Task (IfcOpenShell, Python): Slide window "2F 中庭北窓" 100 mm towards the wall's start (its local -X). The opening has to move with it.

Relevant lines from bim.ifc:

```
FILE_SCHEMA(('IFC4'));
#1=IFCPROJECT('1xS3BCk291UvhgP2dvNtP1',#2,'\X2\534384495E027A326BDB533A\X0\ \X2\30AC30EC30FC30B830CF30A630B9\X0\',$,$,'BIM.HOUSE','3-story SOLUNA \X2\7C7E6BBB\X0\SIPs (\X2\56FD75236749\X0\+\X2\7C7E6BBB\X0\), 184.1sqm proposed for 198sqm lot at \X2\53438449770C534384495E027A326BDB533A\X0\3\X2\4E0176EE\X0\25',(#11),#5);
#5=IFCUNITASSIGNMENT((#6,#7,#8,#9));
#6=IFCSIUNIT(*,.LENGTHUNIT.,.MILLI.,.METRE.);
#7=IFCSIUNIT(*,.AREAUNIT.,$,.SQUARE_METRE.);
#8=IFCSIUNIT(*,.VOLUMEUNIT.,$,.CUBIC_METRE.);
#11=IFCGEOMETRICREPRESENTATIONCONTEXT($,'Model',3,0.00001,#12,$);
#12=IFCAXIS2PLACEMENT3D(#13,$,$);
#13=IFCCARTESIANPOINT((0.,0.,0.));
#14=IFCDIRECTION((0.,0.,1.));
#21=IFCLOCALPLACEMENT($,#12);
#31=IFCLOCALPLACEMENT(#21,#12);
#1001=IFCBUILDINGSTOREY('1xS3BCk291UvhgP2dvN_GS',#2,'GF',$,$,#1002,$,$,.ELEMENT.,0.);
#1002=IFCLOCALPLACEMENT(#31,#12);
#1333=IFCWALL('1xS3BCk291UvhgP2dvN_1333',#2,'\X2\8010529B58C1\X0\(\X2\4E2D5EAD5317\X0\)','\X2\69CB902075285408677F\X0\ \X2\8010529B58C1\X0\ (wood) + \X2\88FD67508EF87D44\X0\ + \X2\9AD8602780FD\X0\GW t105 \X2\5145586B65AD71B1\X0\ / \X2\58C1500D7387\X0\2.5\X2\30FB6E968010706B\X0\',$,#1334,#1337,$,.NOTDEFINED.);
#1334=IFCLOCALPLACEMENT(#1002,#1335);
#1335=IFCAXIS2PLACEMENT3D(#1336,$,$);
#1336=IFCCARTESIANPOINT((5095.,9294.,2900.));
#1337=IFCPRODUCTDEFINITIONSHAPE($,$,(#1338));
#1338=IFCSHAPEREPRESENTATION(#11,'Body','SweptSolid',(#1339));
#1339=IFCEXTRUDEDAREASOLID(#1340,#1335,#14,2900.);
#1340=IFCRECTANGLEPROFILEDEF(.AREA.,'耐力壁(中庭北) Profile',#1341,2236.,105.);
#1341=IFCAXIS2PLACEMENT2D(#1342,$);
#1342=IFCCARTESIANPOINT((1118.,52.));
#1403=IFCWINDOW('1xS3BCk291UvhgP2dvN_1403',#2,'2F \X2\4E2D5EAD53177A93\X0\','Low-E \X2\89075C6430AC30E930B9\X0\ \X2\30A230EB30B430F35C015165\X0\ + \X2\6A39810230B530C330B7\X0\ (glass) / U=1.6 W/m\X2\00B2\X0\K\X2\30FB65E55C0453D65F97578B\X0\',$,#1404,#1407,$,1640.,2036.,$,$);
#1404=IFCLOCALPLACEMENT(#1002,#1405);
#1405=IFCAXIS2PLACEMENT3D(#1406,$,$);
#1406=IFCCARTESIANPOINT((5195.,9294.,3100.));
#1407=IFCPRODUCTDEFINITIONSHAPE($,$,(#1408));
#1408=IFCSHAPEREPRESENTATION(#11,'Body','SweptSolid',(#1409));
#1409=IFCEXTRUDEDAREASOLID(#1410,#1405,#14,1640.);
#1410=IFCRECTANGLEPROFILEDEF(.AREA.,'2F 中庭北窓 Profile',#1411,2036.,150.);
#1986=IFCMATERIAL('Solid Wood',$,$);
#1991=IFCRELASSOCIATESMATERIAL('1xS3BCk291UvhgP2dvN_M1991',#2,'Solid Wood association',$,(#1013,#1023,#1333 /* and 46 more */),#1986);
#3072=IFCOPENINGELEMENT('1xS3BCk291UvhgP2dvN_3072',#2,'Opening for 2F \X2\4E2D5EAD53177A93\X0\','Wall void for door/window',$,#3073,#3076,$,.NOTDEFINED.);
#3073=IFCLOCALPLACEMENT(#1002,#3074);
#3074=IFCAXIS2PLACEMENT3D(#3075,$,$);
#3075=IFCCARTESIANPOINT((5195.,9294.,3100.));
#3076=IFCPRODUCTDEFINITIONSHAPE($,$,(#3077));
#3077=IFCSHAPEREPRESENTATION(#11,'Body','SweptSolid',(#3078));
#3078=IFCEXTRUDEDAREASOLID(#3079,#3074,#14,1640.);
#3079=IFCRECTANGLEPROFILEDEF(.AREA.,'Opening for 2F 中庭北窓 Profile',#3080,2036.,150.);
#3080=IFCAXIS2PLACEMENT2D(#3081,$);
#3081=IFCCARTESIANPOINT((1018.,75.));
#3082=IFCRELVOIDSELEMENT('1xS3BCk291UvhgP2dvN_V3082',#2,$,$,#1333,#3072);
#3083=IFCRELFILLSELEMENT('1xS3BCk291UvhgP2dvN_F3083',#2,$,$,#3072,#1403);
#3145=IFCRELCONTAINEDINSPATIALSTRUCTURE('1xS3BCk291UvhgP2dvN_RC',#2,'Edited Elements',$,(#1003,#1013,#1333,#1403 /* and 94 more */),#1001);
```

```python
import ifcopenshell
import ifcopenshell.api.geometry
import ifcopenshell.util.placement
import ifcopenshell.util.unit

model = ifcopenshell.open("bim.ifc")
unit_scale = ifcopenshell.util.unit.calculate_unit_scale(model)

window = model.by_guid("1xS3BCk291UvhgP2dvN_1403")
opening = window.FillsVoids[0].RelatingOpeningElement
wall = opening.VoidsElements[0].RelatingBuildingElement

wall_matrix = ifcopenshell.util.placement.get_local_placement(wall.ObjectPlacement)
shift = wall_matrix[:3, 0] * -0.1 / unit_scale
before = ifcopenshell.util.placement.get_local_placement(window.ObjectPlacement)[:3, 3].copy()

# The window is not placed relative to its opening, so move both.
for product in (opening, window):
    matrix = ifcopenshell.util.placement.get_local_placement(product.ObjectPlacement)
    matrix[:3, 3] += shift
    ifcopenshell.api.geometry.edit_object_placement(model, product=product, matrix=matrix, is_si=False)

after = ifcopenshell.util.placement.get_local_placement(window.ObjectPlacement)[:3, 3]
print("window moved by", (after - before).round(3) + 0.0)

model.write("bim_updated.ifc")
```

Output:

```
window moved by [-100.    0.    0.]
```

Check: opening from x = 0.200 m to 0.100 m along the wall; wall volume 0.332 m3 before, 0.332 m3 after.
